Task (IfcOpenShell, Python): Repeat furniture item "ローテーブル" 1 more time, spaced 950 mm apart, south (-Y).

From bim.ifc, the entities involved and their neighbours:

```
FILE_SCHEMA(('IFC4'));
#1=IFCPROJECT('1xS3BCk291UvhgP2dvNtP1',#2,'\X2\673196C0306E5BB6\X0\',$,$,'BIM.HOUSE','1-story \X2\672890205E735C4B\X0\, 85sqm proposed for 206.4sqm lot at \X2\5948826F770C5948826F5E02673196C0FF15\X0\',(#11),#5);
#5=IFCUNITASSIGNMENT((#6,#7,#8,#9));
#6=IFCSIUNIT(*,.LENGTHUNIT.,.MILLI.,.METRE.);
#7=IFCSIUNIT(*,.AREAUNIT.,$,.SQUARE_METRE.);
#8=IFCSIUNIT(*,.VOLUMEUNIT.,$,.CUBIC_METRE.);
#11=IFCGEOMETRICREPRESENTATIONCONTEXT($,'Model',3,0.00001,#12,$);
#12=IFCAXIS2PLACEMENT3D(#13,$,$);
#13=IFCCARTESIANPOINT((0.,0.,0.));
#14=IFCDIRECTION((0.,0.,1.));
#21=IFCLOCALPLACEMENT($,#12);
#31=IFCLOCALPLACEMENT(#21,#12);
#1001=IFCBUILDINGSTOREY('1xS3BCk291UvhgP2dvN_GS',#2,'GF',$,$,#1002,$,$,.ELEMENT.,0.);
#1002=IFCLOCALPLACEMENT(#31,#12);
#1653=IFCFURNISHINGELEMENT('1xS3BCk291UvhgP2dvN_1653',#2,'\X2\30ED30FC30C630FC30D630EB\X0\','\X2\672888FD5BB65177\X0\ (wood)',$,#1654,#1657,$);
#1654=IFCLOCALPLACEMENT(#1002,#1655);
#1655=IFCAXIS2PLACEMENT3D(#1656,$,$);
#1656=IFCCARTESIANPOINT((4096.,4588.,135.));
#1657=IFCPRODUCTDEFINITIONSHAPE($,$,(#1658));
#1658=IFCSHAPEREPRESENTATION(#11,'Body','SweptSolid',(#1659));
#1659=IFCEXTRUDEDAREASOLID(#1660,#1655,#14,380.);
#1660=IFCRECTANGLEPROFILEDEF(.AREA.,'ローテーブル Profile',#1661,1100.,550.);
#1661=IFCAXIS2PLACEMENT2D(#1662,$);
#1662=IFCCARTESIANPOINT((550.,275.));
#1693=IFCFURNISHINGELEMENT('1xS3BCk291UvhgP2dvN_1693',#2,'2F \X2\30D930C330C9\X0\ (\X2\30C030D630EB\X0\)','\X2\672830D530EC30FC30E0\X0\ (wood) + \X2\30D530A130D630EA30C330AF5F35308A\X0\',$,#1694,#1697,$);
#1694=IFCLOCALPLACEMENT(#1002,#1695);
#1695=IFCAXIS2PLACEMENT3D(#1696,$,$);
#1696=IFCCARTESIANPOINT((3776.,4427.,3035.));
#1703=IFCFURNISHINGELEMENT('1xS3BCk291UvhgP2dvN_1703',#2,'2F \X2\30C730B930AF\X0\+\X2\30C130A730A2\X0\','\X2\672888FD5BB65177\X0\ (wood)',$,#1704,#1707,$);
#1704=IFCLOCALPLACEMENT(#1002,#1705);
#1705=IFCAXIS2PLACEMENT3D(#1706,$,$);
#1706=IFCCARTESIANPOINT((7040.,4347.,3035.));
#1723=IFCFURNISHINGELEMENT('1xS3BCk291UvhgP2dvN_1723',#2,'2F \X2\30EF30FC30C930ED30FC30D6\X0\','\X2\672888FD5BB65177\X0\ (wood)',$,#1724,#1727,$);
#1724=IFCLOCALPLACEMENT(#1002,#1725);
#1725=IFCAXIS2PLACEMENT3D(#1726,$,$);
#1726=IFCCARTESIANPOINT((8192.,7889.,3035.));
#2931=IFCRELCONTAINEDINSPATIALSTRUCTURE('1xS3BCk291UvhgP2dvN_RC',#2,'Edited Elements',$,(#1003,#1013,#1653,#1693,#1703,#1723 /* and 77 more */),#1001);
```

```python
import numpy as np
import ifcopenshell
import ifcopenshell.api.geometry
import ifcopenshell.api.root
import ifcopenshell.util.element
import ifcopenshell.util.placement

model = ifcopenshell.open("bim.ifc")


def reuse_history(source, copy):
    """copy_class also copies each property set's owner history, people and application; keep the originals."""
    for rel in copy.IsDefinedBy:
        if rel.is_a("IfcRelDefinesByProperties") and (history := rel.RelatingPropertyDefinition.OwnerHistory):
            rel.RelatingPropertyDefinition.OwnerHistory = source.OwnerHistory
            ifcopenshell.util.element.remove_deep2(model, history)


source = model.by_id(1653)
base = ifcopenshell.util.placement.get_local_placement(source.ObjectPlacement)
step = np.array([0.0, -1.0, 0.0]) * 950.0

for i in range(1, 2):
    copy = ifcopenshell.api.root.copy_class(model, product=source)
    copy.Representation = ifcopenshell.util.element.copy_deep(
        model, source.Representation, exclude=["IfcGeometricRepresentationContext", "IfcRepresentationMap"]
    )
    reuse_history(source, copy)
    matrix = base.copy()
    matrix[:3, 3] += i * step
    print("added at", matrix[:3, 3].round(3) + 0.0)
    ifcopenshell.api.geometry.edit_object_placement(model, product=copy, matrix=matrix, is_si=False)

model.write("bim_updated.ifc")
```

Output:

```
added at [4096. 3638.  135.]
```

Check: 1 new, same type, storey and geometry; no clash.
